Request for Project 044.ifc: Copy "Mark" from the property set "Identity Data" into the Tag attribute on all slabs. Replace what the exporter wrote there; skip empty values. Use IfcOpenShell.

First a look at what the model holds.

```python
import ifcopenshell
import ifcopenshell.util.element

model = ifcopenshell.open("Project 044.ifc")
print(model.schema)
slabs = model.by_type("IfcSlab")
print(len(slabs), "slabs")
for e in slabs[:8]:
    source = ifcopenshell.util.element.get_pset(e, "Identity Data", "Mark")
    target = e.Tag
    print(e.id(), repr(source), repr(target), sep=" | ")
```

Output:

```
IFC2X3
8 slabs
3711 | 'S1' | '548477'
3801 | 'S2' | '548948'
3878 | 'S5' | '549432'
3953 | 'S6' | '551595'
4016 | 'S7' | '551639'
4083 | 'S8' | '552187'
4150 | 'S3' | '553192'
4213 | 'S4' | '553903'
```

```python
import ifcopenshell
import ifcopenshell.util.element

model = ifcopenshell.open("Project 044.ifc")

count = 0
for e in model.by_type("IfcSlab"):
    value = ifcopenshell.util.element.get_pset(e, "Identity Data", "Mark")
    current = e.Tag
    if not value or not value.strip() or current == value:
        continue
    e.Tag = value
    count += 1

print(count, "slabs updated")

model.write("Project 044_v2.ifc")
```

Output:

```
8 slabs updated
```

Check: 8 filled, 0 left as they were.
